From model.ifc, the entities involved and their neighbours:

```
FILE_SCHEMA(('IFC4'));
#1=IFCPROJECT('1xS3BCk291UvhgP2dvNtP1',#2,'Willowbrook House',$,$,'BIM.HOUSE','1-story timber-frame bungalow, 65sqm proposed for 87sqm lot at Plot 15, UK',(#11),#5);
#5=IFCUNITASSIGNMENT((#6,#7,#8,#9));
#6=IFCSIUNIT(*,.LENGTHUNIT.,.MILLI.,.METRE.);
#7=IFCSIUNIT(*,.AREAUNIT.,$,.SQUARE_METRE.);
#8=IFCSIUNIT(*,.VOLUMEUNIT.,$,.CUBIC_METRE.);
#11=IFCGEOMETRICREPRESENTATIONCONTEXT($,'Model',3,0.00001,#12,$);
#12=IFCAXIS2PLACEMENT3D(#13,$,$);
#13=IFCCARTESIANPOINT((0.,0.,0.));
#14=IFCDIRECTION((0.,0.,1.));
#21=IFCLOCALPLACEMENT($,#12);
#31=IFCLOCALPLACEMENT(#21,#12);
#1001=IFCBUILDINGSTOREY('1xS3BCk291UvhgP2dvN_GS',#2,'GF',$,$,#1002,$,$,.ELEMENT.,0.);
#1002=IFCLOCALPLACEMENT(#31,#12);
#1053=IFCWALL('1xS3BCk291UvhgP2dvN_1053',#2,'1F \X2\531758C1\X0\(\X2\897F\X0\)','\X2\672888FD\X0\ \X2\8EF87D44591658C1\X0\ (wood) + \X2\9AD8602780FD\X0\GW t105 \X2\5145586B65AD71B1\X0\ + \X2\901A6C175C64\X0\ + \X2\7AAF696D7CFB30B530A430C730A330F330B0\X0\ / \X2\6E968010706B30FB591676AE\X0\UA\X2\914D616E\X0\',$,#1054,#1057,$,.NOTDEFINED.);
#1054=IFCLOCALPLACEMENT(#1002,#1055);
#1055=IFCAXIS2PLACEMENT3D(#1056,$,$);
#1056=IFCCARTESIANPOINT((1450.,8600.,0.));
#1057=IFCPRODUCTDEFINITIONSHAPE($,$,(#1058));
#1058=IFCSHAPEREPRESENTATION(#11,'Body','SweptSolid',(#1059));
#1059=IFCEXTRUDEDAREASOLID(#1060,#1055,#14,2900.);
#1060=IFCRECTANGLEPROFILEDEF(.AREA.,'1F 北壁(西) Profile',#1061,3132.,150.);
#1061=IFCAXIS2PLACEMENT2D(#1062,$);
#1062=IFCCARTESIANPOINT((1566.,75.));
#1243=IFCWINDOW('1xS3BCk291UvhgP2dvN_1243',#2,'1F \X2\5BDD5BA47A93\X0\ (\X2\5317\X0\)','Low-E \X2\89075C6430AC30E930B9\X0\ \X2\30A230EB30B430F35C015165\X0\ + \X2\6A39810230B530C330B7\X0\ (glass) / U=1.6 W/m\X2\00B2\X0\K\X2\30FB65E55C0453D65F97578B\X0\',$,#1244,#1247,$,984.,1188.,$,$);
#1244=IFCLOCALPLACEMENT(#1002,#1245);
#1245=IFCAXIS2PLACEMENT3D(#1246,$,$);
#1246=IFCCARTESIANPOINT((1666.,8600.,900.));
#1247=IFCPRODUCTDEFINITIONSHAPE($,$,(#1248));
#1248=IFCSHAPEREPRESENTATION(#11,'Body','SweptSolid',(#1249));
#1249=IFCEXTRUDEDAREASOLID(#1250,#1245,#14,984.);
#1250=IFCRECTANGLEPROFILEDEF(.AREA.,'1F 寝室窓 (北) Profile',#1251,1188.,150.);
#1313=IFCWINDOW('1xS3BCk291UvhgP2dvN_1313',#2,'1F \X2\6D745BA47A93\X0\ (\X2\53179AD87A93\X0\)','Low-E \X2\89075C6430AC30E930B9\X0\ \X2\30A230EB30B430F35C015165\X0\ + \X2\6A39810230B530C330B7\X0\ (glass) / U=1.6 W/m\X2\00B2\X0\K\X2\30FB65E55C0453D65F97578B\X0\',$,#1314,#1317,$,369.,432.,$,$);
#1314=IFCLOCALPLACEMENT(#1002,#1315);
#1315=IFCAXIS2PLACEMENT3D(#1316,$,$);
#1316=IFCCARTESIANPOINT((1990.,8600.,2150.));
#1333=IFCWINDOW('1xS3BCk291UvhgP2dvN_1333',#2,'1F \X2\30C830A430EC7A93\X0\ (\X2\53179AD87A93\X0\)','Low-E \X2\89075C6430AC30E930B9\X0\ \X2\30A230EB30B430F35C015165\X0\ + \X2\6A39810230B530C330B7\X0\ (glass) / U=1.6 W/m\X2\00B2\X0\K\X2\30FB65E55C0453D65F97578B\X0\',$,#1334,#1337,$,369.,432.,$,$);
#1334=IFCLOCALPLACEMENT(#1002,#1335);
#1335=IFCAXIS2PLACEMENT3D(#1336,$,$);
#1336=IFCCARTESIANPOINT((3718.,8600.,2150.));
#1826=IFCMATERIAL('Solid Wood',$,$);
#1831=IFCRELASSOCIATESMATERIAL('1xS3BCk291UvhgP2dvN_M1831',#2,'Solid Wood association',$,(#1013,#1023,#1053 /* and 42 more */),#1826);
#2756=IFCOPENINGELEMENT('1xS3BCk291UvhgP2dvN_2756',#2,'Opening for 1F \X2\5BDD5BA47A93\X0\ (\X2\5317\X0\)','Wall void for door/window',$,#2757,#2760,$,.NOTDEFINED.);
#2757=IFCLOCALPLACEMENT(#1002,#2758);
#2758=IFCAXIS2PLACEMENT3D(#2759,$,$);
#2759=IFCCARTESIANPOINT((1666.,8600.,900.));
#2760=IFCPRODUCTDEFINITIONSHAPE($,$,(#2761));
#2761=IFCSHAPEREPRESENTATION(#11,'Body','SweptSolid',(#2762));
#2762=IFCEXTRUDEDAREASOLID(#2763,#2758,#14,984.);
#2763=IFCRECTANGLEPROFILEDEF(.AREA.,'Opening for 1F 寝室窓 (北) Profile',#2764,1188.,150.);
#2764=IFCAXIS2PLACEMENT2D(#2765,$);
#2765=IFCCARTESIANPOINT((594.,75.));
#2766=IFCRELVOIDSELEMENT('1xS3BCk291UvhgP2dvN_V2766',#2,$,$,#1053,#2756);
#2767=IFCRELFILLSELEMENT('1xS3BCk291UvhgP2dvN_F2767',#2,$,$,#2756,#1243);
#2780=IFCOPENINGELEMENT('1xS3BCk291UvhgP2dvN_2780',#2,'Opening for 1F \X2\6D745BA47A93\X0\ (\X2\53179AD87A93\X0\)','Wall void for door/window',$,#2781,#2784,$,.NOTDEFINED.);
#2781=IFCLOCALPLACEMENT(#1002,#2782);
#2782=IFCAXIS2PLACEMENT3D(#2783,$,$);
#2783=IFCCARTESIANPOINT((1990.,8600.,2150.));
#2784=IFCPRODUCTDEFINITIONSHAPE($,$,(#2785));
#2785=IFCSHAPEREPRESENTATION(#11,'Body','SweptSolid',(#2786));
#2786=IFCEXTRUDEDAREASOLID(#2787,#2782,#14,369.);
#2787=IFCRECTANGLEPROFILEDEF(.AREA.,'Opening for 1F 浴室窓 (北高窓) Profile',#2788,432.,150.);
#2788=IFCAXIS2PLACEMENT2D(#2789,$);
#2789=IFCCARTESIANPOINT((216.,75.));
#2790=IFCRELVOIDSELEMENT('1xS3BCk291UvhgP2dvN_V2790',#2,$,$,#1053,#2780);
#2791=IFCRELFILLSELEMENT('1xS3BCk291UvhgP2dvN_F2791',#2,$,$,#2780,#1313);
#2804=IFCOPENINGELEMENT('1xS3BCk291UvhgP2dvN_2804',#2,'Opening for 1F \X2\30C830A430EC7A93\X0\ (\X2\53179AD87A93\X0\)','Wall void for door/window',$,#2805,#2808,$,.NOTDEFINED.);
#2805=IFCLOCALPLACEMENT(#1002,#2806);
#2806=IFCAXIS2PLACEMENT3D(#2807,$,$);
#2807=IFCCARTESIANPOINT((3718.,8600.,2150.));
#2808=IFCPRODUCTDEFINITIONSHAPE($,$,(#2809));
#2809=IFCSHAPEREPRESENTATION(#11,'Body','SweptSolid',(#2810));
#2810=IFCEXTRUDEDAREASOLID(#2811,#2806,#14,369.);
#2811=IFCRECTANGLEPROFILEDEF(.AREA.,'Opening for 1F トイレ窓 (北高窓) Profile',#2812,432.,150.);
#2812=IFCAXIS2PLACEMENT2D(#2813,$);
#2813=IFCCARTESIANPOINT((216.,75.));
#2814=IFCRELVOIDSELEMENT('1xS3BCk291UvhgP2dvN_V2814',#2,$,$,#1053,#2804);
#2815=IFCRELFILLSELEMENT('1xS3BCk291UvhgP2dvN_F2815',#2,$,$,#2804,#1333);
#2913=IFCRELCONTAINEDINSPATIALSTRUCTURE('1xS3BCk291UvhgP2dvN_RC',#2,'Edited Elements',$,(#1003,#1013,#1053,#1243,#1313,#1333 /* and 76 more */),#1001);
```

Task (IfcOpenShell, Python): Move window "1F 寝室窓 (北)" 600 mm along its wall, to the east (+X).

```python
import ifcopenshell
import ifcopenshell.api.geometry
import ifcopenshell.util.placement
import ifcopenshell.util.unit

model = ifcopenshell.open("model.ifc")
unit_scale = ifcopenshell.util.unit.calculate_unit_scale(model)

window = model.by_guid("1xS3BCk291UvhgP2dvN_1243")
opening = window.FillsVoids[0].RelatingOpeningElement
wall = opening.VoidsElements[0].RelatingBuildingElement

wall_matrix = ifcopenshell.util.placement.get_local_placement(wall.ObjectPlacement)
shift = wall_matrix[:3, 0] * 0.6 / unit_scale
before = ifcopenshell.util.placement.get_local_placement(window.ObjectPlacement)[:3, 3].copy()

# The window is not placed relative to its opening, so move both.
for product in (opening, window):
    matrix = ifcopenshell.util.placement.get_local_placement(product.ObjectPlacement)
    matrix[:3, 3] += shift
    ifcopenshell.api.geometry.edit_object_placement(model, product=product, matrix=matrix, is_si=False)

after = ifcopenshell.util.placement.get_local_placement(window.ObjectPlacement)[:3, 3]
print("window moved by", (after - before).round(3) + 0.0)

model.write("model_edited.ifc")
```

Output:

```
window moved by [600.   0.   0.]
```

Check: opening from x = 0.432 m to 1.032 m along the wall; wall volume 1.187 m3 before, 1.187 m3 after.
